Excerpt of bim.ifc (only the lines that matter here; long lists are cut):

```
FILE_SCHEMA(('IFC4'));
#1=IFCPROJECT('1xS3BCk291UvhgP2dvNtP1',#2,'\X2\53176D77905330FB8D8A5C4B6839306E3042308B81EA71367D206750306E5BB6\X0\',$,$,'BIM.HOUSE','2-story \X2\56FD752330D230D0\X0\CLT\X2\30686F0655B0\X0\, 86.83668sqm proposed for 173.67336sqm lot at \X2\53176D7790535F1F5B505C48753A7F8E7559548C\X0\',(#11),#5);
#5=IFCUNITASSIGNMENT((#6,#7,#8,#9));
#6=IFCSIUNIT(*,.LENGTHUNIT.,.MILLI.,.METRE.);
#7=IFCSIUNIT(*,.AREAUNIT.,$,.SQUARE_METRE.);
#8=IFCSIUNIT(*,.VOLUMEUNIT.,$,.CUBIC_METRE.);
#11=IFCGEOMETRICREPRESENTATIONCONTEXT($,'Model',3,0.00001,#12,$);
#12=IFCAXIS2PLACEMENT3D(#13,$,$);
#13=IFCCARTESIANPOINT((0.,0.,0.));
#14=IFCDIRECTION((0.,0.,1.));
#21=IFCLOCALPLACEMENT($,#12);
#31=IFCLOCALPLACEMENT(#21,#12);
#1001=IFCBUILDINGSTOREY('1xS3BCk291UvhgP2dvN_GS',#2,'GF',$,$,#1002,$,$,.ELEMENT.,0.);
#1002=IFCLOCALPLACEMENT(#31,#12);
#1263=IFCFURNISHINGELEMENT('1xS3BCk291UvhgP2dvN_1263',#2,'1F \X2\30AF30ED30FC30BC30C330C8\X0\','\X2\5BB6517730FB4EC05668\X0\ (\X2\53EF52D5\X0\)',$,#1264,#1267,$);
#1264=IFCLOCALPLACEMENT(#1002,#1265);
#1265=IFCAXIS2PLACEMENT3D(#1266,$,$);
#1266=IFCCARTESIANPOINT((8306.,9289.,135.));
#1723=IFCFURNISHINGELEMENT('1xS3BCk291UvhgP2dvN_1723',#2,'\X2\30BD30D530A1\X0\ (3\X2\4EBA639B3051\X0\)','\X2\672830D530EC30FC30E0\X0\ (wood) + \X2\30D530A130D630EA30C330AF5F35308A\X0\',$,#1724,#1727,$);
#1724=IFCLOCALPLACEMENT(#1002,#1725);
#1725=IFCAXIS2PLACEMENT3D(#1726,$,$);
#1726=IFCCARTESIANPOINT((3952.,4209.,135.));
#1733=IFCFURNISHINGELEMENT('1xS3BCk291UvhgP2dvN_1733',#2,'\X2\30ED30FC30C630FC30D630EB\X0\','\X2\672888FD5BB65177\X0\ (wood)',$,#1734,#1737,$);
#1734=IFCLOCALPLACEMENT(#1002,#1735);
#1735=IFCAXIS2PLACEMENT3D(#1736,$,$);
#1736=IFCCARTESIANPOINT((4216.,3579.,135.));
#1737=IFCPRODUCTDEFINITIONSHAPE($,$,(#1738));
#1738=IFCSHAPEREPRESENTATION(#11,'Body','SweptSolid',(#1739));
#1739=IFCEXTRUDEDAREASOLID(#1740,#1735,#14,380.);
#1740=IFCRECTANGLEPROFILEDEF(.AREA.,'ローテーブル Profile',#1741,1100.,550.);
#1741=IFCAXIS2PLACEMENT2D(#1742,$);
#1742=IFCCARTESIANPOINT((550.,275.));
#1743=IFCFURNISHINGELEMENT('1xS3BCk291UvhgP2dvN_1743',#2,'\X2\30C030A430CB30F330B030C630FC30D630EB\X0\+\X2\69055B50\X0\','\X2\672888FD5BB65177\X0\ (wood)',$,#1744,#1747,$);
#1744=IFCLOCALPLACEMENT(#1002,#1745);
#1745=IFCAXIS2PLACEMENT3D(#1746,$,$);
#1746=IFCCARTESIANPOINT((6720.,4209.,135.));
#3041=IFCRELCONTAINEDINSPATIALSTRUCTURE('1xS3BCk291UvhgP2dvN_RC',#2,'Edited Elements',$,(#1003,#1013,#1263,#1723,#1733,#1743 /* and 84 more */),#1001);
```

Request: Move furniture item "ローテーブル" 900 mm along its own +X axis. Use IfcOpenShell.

```python
import ifcopenshell
import ifcopenshell.api.geometry
import ifcopenshell.util.placement
import ifcopenshell.util.unit

model = ifcopenshell.open("bim.ifc")
unit_scale = ifcopenshell.util.unit.calculate_unit_scale(model)

item = model.by_id(1733)
matrix = ifcopenshell.util.placement.get_local_placement(item.ObjectPlacement)
matrix[:3, 3] += matrix[:3, 0] * 0.9 / unit_scale
ifcopenshell.api.geometry.edit_object_placement(model, product=item, matrix=matrix, is_si=False)

print(ifcopenshell.util.placement.get_local_placement(item.ObjectPlacement).round(3) + 0.0)

model.write("bim_edited.ifc")
```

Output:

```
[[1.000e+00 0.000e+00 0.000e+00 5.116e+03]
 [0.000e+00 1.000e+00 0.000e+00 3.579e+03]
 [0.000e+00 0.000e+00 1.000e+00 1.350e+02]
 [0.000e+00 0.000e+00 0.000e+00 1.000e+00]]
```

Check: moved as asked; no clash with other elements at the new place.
